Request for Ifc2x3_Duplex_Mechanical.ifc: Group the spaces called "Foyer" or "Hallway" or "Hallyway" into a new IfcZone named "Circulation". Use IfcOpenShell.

First a look at what the model holds.

```python
import ifcopenshell

model = ifcopenshell.open("Ifc2x3_Duplex_Mechanical.ifc")
print(model.schema)
seen = {}
for space in model.by_type("IfcSpace"):
    seen[space.LongName] = seen.get(space.LongName, 0) + 1
for name, count in sorted(seen.items(), key=str):
    print(count, "x", name)
print("zones:", [z.Name for z in model.by_type("IfcZone")][:20])
```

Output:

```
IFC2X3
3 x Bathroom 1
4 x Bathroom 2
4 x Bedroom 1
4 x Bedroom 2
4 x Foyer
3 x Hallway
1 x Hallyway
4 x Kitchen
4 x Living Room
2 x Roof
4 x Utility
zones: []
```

```python
import ifcopenshell
import ifcopenshell.api.group
import ifcopenshell.api.root

model = ifcopenshell.open("Ifc2x3_Duplex_Mechanical.ifc")

names = {"Foyer", "Hallway", "Hallyway"}
spaces = [s for s in model.by_type("IfcSpace") if s.LongName in names]

zone = ifcopenshell.api.root.create_entity(model, ifc_class="IfcZone", name="Circulation")
ifcopenshell.api.group.assign_group(model, products=spaces, group=zone)
print(len(spaces), "spaces in", zone.Name)

model.write("Ifc2x3_Duplex_Mechanical_v2.ifc")
```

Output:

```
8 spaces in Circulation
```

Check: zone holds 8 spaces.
